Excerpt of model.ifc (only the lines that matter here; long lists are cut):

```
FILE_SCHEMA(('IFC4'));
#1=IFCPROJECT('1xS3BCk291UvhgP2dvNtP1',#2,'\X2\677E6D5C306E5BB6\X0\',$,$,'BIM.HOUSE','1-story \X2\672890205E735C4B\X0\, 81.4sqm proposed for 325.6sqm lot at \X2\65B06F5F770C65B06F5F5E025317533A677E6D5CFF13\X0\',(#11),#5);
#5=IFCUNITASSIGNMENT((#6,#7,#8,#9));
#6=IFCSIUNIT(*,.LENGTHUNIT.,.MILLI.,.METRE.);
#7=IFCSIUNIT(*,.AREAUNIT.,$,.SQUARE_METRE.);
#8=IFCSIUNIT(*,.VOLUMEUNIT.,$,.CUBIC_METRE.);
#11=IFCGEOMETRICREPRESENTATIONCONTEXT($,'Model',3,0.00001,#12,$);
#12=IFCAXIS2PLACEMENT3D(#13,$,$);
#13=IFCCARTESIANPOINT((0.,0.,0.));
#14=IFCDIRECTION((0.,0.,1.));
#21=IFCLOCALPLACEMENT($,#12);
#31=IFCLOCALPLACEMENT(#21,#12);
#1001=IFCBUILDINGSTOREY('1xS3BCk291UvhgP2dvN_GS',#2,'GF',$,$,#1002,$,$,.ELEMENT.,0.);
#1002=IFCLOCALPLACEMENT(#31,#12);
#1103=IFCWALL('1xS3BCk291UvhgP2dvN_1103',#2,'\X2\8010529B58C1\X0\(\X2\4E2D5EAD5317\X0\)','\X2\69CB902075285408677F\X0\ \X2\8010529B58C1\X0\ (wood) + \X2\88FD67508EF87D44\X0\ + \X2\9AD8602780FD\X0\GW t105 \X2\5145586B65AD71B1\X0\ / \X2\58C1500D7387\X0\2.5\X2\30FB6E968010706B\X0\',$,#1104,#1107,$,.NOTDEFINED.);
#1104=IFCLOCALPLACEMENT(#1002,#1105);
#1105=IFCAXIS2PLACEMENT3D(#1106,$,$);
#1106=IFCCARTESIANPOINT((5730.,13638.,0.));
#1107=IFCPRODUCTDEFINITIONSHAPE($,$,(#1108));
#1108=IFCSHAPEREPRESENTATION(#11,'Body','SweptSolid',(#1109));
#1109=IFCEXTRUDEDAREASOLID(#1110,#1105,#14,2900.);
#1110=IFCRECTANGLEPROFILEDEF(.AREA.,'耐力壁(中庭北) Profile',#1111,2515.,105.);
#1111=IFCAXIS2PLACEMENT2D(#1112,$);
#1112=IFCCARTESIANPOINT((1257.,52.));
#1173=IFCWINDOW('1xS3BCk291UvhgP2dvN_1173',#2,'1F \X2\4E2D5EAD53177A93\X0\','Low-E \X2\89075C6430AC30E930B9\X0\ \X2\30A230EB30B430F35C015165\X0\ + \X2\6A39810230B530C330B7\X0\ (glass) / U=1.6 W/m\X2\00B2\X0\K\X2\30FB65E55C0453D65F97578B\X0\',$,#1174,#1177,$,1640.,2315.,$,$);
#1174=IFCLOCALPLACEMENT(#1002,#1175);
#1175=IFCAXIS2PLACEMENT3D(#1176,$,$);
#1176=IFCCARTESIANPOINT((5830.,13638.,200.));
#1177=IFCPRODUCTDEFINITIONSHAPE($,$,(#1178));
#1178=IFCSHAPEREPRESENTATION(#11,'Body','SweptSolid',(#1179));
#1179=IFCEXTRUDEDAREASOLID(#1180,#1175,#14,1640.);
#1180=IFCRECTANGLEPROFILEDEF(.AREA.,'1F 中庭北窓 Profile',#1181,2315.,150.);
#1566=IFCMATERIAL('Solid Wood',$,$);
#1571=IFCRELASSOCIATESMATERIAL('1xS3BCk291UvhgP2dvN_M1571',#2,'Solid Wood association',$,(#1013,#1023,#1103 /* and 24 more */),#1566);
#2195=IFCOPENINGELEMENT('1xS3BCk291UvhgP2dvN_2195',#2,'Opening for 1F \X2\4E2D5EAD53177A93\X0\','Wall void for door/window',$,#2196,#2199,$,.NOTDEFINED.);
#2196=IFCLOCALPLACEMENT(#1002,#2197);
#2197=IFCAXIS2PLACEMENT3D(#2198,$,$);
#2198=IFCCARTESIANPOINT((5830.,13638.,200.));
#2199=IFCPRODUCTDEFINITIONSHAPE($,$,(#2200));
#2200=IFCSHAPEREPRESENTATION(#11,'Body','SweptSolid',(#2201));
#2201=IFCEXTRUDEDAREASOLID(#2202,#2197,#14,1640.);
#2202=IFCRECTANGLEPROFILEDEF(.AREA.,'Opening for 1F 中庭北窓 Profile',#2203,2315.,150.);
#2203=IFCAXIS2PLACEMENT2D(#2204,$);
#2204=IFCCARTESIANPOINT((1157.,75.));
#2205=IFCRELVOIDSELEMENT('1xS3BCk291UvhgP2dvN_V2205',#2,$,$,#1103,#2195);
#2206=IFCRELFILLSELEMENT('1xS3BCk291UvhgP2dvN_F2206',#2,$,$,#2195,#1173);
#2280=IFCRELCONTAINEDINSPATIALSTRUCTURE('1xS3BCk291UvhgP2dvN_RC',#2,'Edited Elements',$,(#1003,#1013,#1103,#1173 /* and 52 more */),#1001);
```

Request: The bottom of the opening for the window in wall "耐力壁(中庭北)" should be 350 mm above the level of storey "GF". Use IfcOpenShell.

```python
import numpy as np
import ifcopenshell
import ifcopenshell.api.geometry
import ifcopenshell.geom
import ifcopenshell.util.element
import ifcopenshell.util.placement
import ifcopenshell.util.shape
import ifcopenshell.util.unit

model = ifcopenshell.open("model.ifc")
unit_scale = ifcopenshell.util.unit.calculate_unit_scale(model)

window = model.by_id(1173)
opening = window.FillsVoids[0].RelatingOpeningElement
storey = ifcopenshell.util.element.get_container(window, ifc_class="IfcBuildingStorey")
level = ifcopenshell.util.placement.get_local_placement(storey.ObjectPlacement)[2, 3]

# The opening's origin need not be at the sill, so measure its lowest point.
shape = ifcopenshell.geom.create_shape(ifcopenshell.geom.settings(), opening)
bottom = ifcopenshell.util.shape.get_shape_bottom_elevation(shape, shape.geometry) / unit_scale
dz = level + 350.0 - bottom

shift = np.array([0.0, 0.0, dz])
# The window is not placed relative to its opening, so move both.
for product in (opening, window):
    matrix = ifcopenshell.util.placement.get_local_placement(product.ObjectPlacement)
    matrix[:3, 3] += shift
    ifcopenshell.api.geometry.edit_object_placement(model, product=product, matrix=matrix, is_si=False)

print(f"moved by {dz * unit_scale:+.3f} m")

model.write("model-out.ifc")
```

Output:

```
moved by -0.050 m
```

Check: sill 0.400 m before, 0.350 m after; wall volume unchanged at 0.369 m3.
